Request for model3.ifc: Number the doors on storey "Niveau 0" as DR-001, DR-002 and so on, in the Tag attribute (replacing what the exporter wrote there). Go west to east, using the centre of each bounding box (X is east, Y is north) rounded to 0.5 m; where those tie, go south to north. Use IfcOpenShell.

First a look at what the model holds.

```python
import ifcopenshell
import ifcopenshell.util.element
import ifcopenshell.util.placement

model = ifcopenshell.open("model3.ifc")
print(model.schema)
storey = next(s for s in model.by_type("IfcBuildingStorey") if s.Name == "Niveau 0")
doors = [e for e in ifcopenshell.util.element.get_decomposition(storey) if e.is_a("IfcDoor")]
for e in sorted(doors, key=lambda e: e.id()):
    origin = ifcopenshell.util.placement.get_local_placement(e.ObjectPlacement)[:3, 3]
    print(e.id(), e.Tag, e.Name, origin.round(2) + 0.0, sep=" | ")
```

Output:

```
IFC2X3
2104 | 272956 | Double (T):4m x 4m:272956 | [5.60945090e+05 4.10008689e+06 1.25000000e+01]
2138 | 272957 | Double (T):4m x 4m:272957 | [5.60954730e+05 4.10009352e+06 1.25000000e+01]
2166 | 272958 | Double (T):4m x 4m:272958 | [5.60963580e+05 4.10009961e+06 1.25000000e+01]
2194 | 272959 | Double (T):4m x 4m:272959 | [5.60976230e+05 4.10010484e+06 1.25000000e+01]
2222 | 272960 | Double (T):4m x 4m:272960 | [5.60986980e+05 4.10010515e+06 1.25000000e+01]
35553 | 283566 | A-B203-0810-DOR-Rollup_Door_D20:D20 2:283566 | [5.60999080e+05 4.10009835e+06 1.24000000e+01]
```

```python
import ifcopenshell
import ifcopenshell.geom
import ifcopenshell.util.element
import ifcopenshell.util.shape

model = ifcopenshell.open("model3.ifc")
settings = ifcopenshell.geom.settings()
settings.set("use-world-coords", True)


def centre(element):
    shape = ifcopenshell.geom.create_shape(settings, element)
    return ifcopenshell.util.shape.get_bbox_centroid(shape.geometry)


storey = next(s for s in model.by_type("IfcBuildingStorey") if s.Name == "Niveau 0")
doors = [e for e in ifcopenshell.util.element.get_decomposition(storey) if e.is_a("IfcDoor")]

# Insertion points can sit at a corner or the storey origin, so sort by the geometry (in metres).
centres = {e: centre(e) for e in doors}
doors.sort(key=lambda e: (round(centres[e][0] / 0.5), centres[e][1]))

for i, e in enumerate(doors, start=1):
    number = f"DR-0{i:02d}"
    e.Tag = number
    print(e.id(), number)

model.write("model3_updated.ifc")
```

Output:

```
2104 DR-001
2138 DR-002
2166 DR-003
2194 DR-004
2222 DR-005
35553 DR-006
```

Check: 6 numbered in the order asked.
